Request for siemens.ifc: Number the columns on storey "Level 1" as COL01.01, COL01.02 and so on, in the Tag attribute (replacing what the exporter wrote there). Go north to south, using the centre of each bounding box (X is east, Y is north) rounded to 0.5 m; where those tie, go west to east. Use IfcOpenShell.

First a look at what the model holds.

```python
import ifcopenshell
import ifcopenshell.util.element
import ifcopenshell.util.placement

model = ifcopenshell.open("siemens.ifc")
print(model.schema)
storey = next(s for s in model.by_type("IfcBuildingStorey") if s.Name == "Level 1")
columns = [e for e in ifcopenshell.util.element.get_decomposition(storey) if e.is_a("IfcColumn")]
for e in sorted(columns, key=lambda e: e.id()):
    origin = ifcopenshell.util.placement.get_local_placement(e.ObjectPlacement)[:3, 3]
    print(e.id(), e.Tag, e.Name, origin.round(2) + 0.0, sep=" | ")
```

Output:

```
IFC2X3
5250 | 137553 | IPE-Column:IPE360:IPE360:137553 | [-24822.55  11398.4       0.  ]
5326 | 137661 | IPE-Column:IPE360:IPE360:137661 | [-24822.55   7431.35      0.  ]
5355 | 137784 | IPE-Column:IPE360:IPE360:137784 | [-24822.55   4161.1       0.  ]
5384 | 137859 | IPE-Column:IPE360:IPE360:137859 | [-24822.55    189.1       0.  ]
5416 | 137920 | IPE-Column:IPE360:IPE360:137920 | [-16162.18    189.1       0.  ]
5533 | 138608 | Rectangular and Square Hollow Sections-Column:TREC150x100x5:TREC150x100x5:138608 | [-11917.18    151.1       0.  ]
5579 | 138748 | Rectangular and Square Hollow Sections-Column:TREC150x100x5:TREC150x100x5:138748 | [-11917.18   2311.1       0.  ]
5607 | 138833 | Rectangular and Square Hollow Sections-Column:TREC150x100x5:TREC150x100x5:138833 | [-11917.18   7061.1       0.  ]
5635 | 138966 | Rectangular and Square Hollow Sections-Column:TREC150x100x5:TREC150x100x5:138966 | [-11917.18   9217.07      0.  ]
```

```python
import ifcopenshell
import ifcopenshell.geom
import ifcopenshell.util.element
import ifcopenshell.util.shape

model = ifcopenshell.open("siemens.ifc")
settings = ifcopenshell.geom.settings()
settings.set("use-world-coords", True)


def centre(element):
    shape = ifcopenshell.geom.create_shape(settings, element)
    return ifcopenshell.util.shape.get_bbox_centroid(shape.geometry)


storey = next(s for s in model.by_type("IfcBuildingStorey") if s.Name == "Level 1")
columns = [e for e in ifcopenshell.util.element.get_decomposition(storey) if e.is_a("IfcColumn")]

# Insertion points can sit at a corner or the storey origin, so sort by the geometry (in metres).
centres = {e: centre(e) for e in columns}
columns.sort(key=lambda e: (-round(centres[e][1] / 0.5), centres[e][0]))

for i, e in enumerate(columns, start=1):
    number = f"COL01.{i:02d}"
    e.Tag = number
    print(e.id(), number)

model.write("siemens_updated.ifc")
```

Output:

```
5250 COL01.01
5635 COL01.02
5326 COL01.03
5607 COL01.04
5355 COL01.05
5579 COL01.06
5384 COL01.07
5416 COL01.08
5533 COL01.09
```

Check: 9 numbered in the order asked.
